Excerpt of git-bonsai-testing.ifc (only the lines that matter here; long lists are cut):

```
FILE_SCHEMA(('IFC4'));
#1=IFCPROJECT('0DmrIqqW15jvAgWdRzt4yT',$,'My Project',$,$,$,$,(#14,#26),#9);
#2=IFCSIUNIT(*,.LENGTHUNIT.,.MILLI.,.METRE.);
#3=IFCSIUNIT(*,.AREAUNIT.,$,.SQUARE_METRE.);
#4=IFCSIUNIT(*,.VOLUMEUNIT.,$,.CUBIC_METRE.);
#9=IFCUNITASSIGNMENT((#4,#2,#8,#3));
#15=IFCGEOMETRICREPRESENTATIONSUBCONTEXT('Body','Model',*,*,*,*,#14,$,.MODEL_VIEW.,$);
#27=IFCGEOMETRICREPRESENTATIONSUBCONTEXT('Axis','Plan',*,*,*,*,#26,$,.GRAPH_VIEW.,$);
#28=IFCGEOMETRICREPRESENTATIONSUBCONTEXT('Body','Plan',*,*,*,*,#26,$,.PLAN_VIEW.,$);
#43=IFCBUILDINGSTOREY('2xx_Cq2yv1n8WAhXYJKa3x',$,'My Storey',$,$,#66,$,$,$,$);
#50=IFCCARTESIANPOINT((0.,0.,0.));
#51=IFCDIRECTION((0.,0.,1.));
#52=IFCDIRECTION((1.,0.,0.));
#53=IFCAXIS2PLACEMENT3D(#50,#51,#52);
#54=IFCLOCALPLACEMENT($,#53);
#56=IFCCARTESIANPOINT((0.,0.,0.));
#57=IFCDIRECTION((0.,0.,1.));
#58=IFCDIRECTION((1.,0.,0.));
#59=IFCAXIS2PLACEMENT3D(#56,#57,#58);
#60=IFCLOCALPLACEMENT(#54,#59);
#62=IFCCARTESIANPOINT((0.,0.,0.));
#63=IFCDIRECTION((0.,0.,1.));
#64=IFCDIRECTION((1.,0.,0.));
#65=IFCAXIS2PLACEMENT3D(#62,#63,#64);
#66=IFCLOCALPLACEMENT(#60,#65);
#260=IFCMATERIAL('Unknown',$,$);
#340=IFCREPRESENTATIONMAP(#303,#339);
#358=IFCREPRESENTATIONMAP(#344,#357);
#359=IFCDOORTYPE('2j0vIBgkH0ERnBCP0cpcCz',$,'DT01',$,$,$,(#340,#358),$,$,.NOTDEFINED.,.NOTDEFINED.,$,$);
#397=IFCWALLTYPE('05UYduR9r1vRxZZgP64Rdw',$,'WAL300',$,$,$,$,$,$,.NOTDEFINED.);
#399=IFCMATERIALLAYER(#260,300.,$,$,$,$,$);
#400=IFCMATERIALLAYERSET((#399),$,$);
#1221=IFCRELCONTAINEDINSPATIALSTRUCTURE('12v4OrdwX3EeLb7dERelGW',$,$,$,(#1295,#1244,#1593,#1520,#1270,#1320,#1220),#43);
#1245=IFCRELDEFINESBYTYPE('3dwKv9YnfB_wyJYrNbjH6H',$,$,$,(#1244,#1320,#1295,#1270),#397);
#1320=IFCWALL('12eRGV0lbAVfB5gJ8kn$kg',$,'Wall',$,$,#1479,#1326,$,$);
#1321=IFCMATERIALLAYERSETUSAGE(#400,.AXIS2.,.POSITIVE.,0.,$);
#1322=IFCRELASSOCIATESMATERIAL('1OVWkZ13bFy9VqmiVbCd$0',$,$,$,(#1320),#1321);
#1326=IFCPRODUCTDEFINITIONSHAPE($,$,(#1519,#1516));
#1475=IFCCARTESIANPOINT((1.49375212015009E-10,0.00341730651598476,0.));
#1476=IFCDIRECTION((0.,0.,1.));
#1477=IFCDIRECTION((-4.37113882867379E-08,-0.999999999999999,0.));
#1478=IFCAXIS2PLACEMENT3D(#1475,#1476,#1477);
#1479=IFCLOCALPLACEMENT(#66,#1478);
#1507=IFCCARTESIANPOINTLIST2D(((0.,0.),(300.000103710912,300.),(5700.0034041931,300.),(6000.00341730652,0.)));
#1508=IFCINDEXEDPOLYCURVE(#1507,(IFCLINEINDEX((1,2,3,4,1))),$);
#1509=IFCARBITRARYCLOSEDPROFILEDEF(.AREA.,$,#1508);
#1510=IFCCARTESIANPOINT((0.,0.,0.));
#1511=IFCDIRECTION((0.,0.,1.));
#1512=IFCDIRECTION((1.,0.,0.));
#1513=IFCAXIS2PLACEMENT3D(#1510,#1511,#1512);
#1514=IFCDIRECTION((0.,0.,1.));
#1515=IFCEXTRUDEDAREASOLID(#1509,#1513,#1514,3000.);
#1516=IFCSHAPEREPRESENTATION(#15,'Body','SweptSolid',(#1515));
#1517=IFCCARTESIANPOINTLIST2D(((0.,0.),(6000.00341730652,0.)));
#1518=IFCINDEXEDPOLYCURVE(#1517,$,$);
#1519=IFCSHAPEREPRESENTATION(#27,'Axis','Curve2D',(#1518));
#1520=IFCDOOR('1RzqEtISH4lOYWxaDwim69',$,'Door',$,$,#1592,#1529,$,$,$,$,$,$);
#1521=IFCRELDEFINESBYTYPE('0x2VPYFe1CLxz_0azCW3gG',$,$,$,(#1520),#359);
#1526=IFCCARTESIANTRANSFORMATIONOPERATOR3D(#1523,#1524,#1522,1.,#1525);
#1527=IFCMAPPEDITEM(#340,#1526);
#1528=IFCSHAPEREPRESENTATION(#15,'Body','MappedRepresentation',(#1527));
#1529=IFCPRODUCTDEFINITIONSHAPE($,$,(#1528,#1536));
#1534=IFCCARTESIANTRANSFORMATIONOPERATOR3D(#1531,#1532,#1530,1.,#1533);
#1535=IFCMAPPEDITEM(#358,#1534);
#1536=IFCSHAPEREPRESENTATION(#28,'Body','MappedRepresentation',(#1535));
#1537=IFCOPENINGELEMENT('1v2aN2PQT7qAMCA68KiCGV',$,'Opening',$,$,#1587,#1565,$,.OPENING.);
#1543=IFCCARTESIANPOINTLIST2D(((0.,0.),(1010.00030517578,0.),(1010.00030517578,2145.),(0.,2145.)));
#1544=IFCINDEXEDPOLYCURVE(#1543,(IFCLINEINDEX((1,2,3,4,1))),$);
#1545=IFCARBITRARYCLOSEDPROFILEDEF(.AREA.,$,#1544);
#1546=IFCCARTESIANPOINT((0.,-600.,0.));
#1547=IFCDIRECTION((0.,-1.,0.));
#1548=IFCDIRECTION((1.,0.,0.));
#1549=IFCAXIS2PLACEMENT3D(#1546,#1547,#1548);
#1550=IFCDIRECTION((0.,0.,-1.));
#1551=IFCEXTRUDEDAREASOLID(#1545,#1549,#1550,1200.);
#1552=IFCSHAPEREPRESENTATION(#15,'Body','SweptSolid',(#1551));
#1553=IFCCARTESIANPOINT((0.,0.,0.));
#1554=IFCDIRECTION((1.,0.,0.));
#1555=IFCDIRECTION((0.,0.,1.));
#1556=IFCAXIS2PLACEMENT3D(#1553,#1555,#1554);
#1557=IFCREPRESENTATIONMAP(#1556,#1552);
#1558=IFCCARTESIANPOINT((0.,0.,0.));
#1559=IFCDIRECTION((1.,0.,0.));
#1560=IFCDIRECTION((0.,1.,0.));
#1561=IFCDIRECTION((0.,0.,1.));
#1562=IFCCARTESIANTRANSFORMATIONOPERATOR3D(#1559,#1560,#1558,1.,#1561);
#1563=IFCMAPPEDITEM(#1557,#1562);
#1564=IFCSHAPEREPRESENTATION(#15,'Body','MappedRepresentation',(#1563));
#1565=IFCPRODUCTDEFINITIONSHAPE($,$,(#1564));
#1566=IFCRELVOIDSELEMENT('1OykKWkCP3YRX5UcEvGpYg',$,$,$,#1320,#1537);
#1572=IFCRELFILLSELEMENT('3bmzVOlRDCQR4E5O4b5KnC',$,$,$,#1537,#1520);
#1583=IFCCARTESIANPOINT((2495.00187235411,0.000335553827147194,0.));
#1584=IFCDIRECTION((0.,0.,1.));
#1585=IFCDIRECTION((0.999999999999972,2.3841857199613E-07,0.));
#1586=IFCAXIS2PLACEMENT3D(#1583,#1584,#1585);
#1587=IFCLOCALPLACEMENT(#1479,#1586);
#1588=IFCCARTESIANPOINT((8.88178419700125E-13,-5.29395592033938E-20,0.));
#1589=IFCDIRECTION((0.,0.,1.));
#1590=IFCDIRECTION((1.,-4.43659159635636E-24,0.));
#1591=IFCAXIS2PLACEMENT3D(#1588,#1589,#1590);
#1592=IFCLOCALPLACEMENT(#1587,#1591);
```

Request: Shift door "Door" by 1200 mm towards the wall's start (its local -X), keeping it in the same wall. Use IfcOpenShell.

```python
import ifcopenshell
import ifcopenshell.api.geometry
import ifcopenshell.util.placement

model = ifcopenshell.open("git-bonsai-testing.ifc")

door = model.by_id(1520)
opening = door.FillsVoids[0].RelatingOpeningElement
wall = opening.VoidsElements[0].RelatingBuildingElement

wall_matrix = ifcopenshell.util.placement.get_local_placement(wall.ObjectPlacement)
shift = wall_matrix[:3, 0] * -1200.0
before = ifcopenshell.util.placement.get_local_placement(door.ObjectPlacement)[:3, 3].copy()

# The door is placed relative to its opening, so it follows when the opening moves.
matrix = ifcopenshell.util.placement.get_local_placement(opening.ObjectPlacement)
matrix[:3, 3] += shift
ifcopenshell.api.geometry.edit_object_placement(
    model, product=opening, matrix=matrix, is_si=False, should_transform_children=True
)

after = ifcopenshell.util.placement.get_local_placement(door.ObjectPlacement)[:3, 3]
print("door moved by", (after - before).round(3) + 0.0)

model.write("git-bonsai-testing_rev.ifc")
```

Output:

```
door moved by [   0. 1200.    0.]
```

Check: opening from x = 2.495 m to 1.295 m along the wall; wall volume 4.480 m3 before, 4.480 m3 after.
